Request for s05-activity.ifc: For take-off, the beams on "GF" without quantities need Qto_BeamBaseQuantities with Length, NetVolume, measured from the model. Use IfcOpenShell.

First a look at what the model holds.

```python
import ifcopenshell
import ifcopenshell.util.element
import ifcopenshell.util.unit

model = ifcopenshell.open("s05-activity.ifc")
print(model.schema)
for unit_type in ("LENGTHUNIT", "AREAUNIT", "VOLUMEUNIT"):
    print(unit_type, ifcopenshell.util.unit.calculate_unit_scale(model, unit_type))
storey = next(s for s in model.by_type("IfcBuildingStorey") if s.Name == "GF")
beams = [e for e in ifcopenshell.util.element.get_decomposition(storey) if e.is_a("IfcBeam")]
for e in sorted(beams, key=lambda e: e.id()):
    print(e.id(), e.is_a(), e.Name, list(ifcopenshell.util.element.get_psets(e, qtos_only=True)), sep=" | ")
```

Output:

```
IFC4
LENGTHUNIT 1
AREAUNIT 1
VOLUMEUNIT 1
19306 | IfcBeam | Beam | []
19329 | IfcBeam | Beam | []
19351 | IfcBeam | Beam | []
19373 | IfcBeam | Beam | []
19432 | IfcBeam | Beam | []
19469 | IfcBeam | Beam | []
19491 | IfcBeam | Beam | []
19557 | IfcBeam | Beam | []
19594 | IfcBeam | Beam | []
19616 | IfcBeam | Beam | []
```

```python
import ifcopenshell
import ifcopenshell.api.pset
import ifcopenshell.geom
import ifcopenshell.util.element
import ifcopenshell.util.shape
import ifcopenshell.util.unit

model = ifcopenshell.open("s05-activity.ifc")
unit_scale = ifcopenshell.util.unit.calculate_unit_scale(model)
volume_scale = ifcopenshell.util.unit.calculate_unit_scale(model, "VOLUMEUNIT")
settings = ifcopenshell.geom.settings()

storey = next(s for s in model.by_type("IfcBuildingStorey") if s.Name == "GF")
beams = [e for e in ifcopenshell.util.element.get_decomposition(storey) if e.is_a("IfcBeam")]

for e in sorted(beams, key=lambda e: e.id()):
    if ifcopenshell.util.element.get_psets(e, qtos_only=True, should_inherit=False):
        continue
    # Geometry comes back in metres, in the element's own axes.
    shape = ifcopenshell.geom.create_shape(settings, e)
    values = {
        "Length": ifcopenshell.util.shape.get_max_xyz(shape.geometry) / unit_scale,
        "NetVolume": ifcopenshell.util.shape.get_volume(shape.geometry) / volume_scale,
    }
    qto = ifcopenshell.api.pset.add_qto(model, product=e, name="Qto_BeamBaseQuantities")
    ifcopenshell.api.pset.edit_qto(model, qto=qto, properties=values)
    print(e.id(), {k: round(v, 3) for k, v in values.items()})

model.write("s05-activity_v2.ifc")
```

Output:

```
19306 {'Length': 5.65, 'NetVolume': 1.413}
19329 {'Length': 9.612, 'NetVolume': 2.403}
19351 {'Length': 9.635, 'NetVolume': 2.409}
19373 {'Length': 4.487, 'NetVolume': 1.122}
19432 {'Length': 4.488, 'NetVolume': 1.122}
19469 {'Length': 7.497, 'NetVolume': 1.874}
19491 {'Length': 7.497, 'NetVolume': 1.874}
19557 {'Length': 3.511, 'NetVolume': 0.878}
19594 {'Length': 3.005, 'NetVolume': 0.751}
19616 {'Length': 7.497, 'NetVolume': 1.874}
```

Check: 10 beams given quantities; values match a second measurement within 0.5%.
